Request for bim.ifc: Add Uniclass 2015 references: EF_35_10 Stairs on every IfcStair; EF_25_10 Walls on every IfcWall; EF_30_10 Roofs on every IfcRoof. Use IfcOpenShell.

First a look at what the model holds.

```python
import ifcopenshell

model = ifcopenshell.open("bim.ifc")
print(model.schema)
print("classifications:", [c.Name for c in model.by_type("IfcClassification")])
for ifc_class in ("IfcDoor", "IfcRoof", "IfcStair", "IfcWall", "IfcWindow"):
    print(ifc_class, len(model.by_type(ifc_class)))
```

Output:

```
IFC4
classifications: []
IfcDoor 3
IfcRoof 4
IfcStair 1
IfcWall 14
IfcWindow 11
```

```python
import ifcopenshell
import ifcopenshell.api.classification

model = ifcopenshell.open("bim.ifc")

system = ifcopenshell.api.classification.add_classification(model, classification="Uniclass 2015")

codes = {
    "IfcStair": ("EF_35_10", "Stairs"),
    "IfcWall": ("EF_25_10", "Walls"),
    "IfcRoof": ("EF_30_10", "Roofs"),
}
for ifc_class, (code, name) in codes.items():
    products = model.by_type(ifc_class)
    ifcopenshell.api.classification.add_reference(
        model, products=products, classification=system, identification=code, name=name
    )
    print(code, len(products))

model.write("bim_v2.ifc")
```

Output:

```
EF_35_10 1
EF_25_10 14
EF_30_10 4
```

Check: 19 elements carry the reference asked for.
